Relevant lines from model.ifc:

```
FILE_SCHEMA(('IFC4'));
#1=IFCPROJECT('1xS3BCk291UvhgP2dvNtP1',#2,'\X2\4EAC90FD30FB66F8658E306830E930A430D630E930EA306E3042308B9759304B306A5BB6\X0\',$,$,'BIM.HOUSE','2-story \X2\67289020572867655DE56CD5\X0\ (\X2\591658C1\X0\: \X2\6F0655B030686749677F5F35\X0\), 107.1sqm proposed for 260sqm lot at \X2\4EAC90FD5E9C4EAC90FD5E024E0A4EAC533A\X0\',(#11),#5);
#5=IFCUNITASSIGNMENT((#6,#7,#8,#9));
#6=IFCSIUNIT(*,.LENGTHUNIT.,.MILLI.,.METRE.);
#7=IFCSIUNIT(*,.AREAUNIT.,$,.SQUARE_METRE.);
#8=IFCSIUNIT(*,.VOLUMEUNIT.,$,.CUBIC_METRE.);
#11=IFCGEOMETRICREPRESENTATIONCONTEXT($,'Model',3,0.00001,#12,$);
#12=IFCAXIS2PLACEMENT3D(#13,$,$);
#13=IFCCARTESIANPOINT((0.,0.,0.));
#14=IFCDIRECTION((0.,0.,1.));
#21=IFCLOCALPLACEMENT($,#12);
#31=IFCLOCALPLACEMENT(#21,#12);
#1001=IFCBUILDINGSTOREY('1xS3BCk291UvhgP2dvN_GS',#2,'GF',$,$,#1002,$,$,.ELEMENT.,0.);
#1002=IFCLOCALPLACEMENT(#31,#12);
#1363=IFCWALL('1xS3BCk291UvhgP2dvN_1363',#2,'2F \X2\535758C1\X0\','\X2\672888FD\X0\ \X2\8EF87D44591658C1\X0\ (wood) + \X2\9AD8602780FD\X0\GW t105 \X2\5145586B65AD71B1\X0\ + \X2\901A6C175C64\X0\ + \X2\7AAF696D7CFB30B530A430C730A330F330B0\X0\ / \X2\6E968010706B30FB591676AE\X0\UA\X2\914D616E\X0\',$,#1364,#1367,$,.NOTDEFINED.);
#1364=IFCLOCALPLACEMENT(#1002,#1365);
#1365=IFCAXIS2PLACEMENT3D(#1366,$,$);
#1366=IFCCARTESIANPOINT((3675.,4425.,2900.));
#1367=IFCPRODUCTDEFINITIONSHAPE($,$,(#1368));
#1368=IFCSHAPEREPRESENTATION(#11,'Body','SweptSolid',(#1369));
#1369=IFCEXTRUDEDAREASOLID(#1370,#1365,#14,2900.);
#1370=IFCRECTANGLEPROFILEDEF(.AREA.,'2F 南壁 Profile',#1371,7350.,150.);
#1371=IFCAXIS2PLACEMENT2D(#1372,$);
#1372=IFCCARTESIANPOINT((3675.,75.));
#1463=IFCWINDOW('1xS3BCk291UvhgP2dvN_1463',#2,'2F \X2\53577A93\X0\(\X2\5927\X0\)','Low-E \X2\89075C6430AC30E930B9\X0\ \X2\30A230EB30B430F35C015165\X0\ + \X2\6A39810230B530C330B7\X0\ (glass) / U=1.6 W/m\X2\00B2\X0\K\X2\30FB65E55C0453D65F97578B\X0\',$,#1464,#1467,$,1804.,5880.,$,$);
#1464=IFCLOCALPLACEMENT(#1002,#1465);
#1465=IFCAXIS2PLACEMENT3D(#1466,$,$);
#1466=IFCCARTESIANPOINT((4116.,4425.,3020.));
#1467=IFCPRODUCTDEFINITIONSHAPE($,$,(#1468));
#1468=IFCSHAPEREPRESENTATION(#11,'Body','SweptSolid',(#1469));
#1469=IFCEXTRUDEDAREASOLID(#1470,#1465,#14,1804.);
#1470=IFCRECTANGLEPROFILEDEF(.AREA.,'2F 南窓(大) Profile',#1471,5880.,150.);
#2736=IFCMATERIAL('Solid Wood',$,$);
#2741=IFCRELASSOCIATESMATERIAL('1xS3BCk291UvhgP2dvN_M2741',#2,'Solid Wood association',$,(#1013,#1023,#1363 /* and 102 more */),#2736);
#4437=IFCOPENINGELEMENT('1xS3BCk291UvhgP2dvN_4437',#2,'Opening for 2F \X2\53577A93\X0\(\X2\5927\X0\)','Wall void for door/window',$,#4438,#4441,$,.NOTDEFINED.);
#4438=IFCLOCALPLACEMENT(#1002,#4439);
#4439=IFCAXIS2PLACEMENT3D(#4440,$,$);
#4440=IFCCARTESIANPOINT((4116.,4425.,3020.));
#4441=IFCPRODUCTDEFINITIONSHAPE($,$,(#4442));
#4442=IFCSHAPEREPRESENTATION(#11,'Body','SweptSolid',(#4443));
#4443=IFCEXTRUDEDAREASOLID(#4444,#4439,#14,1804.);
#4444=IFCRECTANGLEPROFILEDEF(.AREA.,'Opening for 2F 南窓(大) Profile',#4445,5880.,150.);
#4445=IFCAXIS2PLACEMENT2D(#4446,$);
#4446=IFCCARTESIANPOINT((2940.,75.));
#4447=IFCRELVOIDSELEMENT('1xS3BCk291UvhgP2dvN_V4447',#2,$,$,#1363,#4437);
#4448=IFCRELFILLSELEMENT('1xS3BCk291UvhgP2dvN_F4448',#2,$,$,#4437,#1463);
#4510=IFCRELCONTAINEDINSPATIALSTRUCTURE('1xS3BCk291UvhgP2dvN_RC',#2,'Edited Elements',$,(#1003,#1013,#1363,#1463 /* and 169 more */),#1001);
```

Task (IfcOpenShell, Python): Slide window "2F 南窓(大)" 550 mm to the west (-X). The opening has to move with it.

```python
import ifcopenshell
import ifcopenshell.api.geometry
import ifcopenshell.util.placement

model = ifcopenshell.open("model.ifc")

window = model.by_guid("1xS3BCk291UvhgP2dvN_1463")
opening = window.FillsVoids[0].RelatingOpeningElement
wall = opening.VoidsElements[0].RelatingBuildingElement

wall_matrix = ifcopenshell.util.placement.get_local_placement(wall.ObjectPlacement)
shift = wall_matrix[:3, 0] * -550.0
before = ifcopenshell.util.placement.get_local_placement(window.ObjectPlacement)[:3, 3].copy()

# The window is not placed relative to its opening, so move both.
for product in (opening, window):
    matrix = ifcopenshell.util.placement.get_local_placement(product.ObjectPlacement)
    matrix[:3, 3] += shift
    ifcopenshell.api.geometry.edit_object_placement(model, product=product, matrix=matrix, is_si=False)

after = ifcopenshell.util.placement.get_local_placement(window.ObjectPlacement)[:3, 3]
print("window moved by", (after - before).round(3) + 0.0)

model.write("model-out.ifc")
```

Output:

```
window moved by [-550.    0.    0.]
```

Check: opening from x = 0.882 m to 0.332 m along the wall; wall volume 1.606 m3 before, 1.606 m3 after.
